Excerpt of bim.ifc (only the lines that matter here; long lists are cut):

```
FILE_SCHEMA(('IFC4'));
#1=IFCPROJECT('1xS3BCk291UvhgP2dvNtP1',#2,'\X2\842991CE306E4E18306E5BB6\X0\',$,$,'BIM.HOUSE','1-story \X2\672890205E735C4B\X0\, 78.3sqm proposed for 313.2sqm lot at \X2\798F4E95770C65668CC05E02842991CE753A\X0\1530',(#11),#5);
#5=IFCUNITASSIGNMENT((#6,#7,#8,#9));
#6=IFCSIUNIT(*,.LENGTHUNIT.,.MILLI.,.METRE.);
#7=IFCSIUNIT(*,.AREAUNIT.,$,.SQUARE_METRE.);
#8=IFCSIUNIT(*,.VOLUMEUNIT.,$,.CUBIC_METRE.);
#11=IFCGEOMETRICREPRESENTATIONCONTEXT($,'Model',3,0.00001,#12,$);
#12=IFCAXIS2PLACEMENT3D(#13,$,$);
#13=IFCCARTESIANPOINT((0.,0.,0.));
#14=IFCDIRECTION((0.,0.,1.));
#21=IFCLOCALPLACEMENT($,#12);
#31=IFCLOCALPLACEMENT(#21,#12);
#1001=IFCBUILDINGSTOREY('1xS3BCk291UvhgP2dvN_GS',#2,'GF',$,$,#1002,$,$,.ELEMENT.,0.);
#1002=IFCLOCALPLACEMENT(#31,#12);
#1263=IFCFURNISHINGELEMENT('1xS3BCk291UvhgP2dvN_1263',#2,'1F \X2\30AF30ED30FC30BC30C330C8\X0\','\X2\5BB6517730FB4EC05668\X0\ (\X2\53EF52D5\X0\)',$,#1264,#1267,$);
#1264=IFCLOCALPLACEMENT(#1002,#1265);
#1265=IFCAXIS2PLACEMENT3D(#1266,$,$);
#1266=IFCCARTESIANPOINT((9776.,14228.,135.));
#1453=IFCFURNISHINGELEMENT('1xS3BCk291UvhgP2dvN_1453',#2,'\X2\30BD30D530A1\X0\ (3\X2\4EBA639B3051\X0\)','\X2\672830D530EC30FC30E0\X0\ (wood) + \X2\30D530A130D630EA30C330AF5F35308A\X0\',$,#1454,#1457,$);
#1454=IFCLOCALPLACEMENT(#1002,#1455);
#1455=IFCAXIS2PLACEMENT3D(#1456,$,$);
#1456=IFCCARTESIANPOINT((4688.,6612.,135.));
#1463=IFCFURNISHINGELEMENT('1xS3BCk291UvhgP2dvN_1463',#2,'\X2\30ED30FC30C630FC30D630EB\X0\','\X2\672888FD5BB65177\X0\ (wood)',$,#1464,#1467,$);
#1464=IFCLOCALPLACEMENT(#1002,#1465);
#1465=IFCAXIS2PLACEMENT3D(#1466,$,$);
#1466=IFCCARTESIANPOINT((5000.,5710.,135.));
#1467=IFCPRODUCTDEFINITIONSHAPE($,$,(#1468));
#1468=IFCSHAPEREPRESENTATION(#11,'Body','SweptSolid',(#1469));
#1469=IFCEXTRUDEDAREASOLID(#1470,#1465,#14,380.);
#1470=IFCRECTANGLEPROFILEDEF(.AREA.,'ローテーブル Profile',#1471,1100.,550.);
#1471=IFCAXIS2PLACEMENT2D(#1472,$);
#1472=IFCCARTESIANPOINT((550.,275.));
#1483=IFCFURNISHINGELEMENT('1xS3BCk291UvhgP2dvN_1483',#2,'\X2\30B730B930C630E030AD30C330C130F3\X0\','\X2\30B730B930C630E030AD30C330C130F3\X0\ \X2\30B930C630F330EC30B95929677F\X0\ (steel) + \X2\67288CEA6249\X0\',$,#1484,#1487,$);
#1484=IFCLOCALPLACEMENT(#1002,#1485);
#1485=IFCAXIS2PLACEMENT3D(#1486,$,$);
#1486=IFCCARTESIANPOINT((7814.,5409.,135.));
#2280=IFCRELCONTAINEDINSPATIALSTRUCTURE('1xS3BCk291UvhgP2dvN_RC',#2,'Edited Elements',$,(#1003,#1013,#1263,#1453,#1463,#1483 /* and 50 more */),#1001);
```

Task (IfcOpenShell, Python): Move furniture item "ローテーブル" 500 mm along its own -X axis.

```python
import ifcopenshell
import ifcopenshell.api.geometry
import ifcopenshell.util.placement

model = ifcopenshell.open("bim.ifc")

item = model.by_id(1463)
matrix = ifcopenshell.util.placement.get_local_placement(item.ObjectPlacement)
matrix[:3, 3] -= matrix[:3, 0] * 500.0
ifcopenshell.api.geometry.edit_object_placement(model, product=item, matrix=matrix, is_si=False)

print(ifcopenshell.util.placement.get_local_placement(item.ObjectPlacement).round(3) + 0.0)

model.write("bim_updated.ifc")
```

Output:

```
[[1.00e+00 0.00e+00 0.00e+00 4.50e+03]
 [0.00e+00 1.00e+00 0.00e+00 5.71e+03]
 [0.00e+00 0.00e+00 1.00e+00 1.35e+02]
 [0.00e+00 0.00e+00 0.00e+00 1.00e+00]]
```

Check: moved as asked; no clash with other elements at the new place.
